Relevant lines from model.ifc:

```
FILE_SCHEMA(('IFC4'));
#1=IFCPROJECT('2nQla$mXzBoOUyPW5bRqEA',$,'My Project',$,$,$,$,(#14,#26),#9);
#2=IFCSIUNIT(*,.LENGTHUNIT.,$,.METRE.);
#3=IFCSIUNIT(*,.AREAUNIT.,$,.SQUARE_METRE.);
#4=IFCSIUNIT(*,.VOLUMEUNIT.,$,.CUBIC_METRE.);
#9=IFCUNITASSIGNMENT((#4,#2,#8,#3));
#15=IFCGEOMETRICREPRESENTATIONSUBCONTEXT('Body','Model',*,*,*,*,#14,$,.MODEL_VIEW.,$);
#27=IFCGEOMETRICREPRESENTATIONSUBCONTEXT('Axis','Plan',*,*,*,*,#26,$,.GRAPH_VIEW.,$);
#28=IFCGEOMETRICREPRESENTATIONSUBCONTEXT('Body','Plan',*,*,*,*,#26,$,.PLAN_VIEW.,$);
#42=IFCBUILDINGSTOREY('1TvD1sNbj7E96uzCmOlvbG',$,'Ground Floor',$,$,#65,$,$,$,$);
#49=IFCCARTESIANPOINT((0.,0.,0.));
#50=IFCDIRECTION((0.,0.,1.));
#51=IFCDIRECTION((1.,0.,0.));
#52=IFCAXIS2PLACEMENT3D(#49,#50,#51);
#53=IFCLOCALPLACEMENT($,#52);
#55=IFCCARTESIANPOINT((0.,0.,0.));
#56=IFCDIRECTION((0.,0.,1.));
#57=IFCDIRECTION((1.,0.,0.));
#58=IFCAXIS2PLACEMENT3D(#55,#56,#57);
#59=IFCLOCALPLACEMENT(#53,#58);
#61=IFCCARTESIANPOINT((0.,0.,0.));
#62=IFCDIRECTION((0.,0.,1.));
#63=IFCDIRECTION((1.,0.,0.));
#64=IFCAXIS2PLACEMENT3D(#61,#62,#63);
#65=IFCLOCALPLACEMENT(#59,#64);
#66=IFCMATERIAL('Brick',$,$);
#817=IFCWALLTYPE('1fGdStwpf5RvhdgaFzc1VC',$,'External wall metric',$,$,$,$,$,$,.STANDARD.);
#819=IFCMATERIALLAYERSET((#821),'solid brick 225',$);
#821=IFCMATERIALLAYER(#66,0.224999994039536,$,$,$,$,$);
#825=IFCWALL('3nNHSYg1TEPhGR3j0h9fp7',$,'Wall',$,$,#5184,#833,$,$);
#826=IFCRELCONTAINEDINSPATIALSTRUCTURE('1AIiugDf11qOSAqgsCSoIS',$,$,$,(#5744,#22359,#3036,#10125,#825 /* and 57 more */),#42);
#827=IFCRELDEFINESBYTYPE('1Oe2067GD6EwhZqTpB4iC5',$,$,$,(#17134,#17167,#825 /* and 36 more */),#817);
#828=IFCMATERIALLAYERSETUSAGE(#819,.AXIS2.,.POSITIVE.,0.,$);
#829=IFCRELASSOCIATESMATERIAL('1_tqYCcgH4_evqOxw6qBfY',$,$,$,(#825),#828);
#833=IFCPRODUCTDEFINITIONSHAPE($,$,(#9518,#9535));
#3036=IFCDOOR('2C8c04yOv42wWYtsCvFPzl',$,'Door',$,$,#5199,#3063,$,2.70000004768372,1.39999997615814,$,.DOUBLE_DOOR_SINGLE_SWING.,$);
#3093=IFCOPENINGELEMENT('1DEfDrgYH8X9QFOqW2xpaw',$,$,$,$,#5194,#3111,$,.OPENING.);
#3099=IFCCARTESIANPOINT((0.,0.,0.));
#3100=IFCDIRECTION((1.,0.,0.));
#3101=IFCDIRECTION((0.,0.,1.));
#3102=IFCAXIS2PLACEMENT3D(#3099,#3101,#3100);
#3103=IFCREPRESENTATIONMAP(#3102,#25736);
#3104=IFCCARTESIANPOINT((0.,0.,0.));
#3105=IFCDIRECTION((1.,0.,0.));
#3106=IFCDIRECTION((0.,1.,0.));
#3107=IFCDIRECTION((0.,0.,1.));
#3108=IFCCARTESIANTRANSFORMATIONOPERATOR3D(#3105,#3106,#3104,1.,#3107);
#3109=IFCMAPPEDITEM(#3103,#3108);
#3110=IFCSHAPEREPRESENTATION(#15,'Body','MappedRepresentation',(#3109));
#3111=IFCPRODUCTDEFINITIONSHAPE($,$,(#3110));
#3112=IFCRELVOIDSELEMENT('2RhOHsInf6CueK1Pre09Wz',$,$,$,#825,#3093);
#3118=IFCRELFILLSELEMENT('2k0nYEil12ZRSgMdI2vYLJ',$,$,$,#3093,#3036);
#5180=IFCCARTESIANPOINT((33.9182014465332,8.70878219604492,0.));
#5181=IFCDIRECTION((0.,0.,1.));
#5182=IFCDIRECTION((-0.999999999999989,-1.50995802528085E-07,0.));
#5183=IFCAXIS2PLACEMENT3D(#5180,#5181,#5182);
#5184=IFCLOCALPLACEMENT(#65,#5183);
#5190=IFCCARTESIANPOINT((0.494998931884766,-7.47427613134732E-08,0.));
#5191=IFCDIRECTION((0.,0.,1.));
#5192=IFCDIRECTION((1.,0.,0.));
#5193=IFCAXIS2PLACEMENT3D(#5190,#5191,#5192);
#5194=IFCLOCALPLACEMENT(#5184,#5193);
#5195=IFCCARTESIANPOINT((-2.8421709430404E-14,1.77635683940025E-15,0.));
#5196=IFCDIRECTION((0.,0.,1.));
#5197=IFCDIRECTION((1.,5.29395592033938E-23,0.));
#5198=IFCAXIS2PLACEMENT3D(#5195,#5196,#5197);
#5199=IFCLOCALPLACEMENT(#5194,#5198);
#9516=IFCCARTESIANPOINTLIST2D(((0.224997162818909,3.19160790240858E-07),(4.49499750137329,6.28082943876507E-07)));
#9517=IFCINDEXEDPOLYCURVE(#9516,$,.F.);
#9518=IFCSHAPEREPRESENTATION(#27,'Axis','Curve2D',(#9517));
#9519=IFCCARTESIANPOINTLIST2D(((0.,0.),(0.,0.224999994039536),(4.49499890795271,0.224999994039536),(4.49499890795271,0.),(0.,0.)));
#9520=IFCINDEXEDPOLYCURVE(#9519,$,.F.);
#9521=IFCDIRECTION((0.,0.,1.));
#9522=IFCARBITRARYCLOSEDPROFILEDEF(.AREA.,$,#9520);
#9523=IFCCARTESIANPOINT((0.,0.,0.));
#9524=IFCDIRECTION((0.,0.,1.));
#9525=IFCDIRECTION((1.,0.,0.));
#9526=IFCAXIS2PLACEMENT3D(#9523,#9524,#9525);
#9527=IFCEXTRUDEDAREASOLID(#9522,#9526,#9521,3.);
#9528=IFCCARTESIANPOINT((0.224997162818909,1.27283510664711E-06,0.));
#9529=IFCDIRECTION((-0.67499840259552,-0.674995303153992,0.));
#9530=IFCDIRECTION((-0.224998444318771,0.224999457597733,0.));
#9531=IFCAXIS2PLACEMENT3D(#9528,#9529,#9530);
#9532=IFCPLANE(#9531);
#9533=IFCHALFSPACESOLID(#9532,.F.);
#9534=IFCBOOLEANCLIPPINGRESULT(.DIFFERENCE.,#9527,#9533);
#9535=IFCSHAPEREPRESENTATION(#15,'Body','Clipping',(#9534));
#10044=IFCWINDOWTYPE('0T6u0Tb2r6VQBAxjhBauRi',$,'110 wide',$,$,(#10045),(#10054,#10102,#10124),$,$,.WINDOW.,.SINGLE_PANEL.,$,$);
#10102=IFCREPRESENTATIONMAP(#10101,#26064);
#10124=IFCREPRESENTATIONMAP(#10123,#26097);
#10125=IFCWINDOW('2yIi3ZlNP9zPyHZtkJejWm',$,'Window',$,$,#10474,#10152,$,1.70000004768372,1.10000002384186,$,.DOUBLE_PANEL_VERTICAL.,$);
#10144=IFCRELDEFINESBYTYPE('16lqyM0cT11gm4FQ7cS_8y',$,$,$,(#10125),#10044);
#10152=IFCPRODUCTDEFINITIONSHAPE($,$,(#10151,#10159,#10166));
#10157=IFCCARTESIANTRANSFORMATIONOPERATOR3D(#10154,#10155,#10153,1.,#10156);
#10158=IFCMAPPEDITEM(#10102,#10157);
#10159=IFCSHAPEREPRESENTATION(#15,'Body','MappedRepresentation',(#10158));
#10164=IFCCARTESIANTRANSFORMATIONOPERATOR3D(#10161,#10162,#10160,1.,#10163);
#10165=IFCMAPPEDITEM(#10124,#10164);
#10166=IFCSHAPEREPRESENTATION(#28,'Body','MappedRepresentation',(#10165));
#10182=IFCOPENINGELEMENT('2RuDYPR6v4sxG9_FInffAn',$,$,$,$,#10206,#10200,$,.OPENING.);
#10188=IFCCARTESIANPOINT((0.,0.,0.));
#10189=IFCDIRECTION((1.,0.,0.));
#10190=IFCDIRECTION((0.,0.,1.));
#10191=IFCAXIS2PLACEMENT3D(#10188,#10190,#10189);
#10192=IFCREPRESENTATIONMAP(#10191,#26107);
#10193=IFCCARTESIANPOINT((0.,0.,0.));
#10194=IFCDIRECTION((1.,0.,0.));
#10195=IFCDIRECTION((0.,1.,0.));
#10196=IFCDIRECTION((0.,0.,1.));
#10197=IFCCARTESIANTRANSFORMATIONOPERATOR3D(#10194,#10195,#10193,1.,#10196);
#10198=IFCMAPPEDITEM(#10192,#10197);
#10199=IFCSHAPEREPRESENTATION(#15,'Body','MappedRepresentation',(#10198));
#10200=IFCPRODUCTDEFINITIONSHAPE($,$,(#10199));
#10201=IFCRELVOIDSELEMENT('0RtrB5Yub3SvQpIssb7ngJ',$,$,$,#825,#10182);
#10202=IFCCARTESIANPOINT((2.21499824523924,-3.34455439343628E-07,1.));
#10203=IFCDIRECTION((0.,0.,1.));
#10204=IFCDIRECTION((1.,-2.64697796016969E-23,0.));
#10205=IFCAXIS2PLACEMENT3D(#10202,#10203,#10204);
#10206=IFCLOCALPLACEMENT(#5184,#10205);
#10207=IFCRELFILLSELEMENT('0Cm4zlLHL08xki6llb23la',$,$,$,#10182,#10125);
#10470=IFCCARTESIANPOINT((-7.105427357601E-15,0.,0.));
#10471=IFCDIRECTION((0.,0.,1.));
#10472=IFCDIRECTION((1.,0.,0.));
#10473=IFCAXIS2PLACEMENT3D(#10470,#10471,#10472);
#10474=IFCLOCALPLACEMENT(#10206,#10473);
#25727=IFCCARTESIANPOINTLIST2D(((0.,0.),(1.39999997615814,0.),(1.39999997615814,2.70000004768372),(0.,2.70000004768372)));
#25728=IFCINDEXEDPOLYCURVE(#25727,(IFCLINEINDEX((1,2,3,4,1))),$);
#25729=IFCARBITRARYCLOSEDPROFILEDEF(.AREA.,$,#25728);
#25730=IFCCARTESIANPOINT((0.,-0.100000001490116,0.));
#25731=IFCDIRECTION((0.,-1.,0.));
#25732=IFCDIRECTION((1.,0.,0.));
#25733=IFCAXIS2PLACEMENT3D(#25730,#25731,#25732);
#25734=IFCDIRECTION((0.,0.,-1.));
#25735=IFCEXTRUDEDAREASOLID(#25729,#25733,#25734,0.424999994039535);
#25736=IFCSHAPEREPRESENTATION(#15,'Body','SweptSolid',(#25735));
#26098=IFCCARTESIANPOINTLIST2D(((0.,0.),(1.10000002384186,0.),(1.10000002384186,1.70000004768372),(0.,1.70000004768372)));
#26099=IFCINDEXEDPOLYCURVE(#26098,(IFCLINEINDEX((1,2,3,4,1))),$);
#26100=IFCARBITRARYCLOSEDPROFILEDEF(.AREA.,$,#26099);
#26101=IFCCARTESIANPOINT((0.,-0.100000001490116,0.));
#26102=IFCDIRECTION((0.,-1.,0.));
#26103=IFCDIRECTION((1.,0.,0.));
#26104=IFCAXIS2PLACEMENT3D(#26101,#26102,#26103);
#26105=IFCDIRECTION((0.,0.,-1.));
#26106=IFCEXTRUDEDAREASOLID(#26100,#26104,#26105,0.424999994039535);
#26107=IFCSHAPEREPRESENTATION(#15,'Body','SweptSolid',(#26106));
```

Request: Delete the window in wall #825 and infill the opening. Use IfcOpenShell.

```python
import ifcopenshell
import ifcopenshell.api.feature
import ifcopenshell.api.root
import ifcopenshell.geom
import ifcopenshell.util.shape

model = ifcopenshell.open("model.ifc")
settings = ifcopenshell.geom.settings()


def volume(element):
    """Net volume in cubic metres, openings subtracted."""
    shape = ifcopenshell.geom.create_shape(settings, element)
    return ifcopenshell.util.shape.get_volume(shape.geometry)


window = model.by_guid("2yIi3ZlNP9zPyHZtkJejWm")
opening = window.FillsVoids[0].RelatingOpeningElement
wall = opening.VoidsElements[0].RelatingBuildingElement
before = volume(wall)

ifcopenshell.api.root.remove_product(model, product=window)
ifcopenshell.api.feature.remove_feature(model, feature=opening)

after = volume(wall)

print(f"wall volume {before:.3f} -> {after:.3f} m3")

model.write("model_rev.ifc")
```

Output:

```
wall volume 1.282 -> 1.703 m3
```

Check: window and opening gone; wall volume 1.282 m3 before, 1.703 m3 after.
